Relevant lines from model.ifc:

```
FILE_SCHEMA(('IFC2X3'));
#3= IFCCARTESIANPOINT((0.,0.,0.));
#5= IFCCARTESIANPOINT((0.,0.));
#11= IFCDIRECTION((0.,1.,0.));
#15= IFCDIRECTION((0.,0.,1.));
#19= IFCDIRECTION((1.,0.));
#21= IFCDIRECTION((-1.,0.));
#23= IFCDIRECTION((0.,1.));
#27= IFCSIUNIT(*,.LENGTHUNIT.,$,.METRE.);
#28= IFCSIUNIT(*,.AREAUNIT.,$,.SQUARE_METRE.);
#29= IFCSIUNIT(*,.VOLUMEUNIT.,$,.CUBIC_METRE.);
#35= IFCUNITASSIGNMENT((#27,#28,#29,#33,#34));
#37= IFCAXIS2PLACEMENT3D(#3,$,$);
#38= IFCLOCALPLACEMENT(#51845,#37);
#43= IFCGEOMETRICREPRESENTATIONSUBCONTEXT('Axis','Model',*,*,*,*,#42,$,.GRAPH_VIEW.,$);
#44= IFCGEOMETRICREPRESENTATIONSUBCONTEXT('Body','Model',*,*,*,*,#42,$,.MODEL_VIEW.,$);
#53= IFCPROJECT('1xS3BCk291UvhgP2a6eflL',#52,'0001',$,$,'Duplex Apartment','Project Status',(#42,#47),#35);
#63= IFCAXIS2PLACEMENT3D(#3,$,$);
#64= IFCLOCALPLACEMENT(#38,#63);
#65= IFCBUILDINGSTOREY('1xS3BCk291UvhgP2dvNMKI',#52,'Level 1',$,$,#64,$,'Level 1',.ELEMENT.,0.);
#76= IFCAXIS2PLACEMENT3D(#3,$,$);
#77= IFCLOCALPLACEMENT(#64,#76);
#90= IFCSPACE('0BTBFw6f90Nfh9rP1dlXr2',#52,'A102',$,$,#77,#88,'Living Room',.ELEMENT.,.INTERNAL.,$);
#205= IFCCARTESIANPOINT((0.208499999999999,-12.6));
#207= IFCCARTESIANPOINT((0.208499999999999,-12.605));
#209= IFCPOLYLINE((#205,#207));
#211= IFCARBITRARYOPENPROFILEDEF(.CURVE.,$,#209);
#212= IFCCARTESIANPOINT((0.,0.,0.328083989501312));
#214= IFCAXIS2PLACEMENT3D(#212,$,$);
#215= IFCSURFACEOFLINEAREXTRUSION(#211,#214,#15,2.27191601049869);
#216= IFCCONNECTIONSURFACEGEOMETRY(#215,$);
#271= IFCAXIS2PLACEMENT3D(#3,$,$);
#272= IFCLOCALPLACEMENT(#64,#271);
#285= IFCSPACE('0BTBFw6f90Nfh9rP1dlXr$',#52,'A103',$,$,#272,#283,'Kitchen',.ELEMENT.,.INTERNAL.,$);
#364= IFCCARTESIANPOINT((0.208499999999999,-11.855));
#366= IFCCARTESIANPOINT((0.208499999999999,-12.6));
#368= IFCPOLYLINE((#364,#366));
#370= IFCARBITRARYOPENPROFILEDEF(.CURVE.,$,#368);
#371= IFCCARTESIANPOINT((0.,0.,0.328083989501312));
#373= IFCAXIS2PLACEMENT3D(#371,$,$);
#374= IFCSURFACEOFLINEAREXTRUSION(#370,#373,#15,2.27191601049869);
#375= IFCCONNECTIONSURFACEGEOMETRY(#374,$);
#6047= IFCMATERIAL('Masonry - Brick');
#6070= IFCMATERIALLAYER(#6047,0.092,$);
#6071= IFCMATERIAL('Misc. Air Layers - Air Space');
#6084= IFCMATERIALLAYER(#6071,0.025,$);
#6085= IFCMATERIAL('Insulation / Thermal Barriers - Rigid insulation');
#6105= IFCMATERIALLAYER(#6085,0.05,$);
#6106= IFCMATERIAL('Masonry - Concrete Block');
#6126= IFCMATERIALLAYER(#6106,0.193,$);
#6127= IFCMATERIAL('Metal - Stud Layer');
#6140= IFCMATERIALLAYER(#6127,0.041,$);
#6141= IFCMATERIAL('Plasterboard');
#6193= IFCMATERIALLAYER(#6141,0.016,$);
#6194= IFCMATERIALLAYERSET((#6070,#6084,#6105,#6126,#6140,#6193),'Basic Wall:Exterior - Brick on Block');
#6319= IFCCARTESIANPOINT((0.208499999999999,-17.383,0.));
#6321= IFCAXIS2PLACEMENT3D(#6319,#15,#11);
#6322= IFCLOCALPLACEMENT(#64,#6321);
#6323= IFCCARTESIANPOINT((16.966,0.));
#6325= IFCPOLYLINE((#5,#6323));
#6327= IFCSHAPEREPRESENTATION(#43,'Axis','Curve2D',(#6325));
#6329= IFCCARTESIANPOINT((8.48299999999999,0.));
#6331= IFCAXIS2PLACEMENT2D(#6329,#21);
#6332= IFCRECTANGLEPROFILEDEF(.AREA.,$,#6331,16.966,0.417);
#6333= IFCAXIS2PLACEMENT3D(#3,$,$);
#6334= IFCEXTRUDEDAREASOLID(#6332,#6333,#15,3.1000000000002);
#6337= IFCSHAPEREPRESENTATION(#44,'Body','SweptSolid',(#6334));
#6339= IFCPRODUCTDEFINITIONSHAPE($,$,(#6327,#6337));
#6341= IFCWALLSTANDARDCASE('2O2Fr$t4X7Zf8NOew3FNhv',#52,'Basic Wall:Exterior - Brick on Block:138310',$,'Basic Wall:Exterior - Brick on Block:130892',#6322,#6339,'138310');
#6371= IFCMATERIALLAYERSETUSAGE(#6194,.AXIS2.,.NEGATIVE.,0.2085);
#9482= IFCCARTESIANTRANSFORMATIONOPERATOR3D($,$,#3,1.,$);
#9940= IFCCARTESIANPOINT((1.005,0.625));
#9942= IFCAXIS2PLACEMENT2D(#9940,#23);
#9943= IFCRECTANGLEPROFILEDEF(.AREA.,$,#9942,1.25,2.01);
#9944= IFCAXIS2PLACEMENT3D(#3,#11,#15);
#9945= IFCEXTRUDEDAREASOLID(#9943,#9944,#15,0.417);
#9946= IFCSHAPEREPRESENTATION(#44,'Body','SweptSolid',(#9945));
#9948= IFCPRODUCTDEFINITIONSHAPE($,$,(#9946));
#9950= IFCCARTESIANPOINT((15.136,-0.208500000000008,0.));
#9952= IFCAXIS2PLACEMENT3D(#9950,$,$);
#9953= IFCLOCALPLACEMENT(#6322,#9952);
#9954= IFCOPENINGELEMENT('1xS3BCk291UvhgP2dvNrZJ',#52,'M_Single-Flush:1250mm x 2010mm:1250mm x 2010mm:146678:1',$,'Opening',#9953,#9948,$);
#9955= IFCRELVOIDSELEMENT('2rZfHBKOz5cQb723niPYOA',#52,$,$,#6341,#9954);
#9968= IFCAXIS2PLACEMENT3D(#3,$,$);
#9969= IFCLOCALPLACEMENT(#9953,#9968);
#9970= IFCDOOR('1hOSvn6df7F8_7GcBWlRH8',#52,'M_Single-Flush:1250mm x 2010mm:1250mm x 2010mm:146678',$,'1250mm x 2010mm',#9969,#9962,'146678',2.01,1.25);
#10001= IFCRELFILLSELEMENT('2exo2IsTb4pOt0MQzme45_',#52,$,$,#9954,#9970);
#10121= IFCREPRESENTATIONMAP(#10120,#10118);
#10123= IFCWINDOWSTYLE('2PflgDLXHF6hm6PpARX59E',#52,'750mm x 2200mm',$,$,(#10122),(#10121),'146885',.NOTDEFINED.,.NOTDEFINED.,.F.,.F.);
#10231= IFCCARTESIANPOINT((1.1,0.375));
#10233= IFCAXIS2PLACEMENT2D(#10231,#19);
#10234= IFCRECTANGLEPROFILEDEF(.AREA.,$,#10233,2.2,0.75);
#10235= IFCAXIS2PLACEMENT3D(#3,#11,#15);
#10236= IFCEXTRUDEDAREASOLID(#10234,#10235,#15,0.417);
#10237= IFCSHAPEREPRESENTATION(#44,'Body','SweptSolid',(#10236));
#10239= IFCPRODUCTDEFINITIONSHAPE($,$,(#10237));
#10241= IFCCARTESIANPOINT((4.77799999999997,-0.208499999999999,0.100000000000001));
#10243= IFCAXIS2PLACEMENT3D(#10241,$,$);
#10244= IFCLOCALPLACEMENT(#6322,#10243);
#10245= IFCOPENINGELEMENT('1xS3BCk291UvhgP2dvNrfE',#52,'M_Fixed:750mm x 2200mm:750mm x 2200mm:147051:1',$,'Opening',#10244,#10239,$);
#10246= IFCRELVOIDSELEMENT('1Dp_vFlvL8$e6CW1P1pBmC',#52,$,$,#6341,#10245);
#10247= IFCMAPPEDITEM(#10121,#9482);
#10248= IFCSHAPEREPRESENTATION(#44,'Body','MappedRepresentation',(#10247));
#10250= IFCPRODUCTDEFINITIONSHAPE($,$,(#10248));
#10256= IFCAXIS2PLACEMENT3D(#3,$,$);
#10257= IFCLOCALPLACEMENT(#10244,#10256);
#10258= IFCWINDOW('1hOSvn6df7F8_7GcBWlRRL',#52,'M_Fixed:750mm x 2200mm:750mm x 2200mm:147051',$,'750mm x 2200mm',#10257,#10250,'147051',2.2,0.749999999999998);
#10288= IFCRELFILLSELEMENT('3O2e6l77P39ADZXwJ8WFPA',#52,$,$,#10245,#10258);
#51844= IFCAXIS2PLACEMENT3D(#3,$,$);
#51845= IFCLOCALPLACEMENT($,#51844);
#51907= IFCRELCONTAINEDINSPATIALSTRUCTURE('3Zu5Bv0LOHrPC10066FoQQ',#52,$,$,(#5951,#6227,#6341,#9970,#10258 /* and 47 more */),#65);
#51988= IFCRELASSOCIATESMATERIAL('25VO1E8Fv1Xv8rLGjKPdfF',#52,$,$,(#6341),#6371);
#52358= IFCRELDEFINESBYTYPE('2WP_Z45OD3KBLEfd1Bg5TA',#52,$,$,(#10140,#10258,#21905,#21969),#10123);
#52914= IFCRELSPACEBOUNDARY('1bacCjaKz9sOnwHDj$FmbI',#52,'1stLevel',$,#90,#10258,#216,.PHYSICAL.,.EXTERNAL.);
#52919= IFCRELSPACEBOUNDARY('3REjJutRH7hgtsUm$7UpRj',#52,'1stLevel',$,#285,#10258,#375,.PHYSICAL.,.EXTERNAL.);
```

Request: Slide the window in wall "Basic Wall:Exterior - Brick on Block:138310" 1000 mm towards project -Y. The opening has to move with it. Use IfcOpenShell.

```python
import numpy as np
import ifcopenshell
import ifcopenshell.api.geometry
import ifcopenshell.util.placement
import ifcopenshell.util.unit

model = ifcopenshell.open("model.ifc")
unit_scale = ifcopenshell.util.unit.calculate_unit_scale(model)

window = model.by_guid("1hOSvn6df7F8_7GcBWlRRL")
opening = window.FillsVoids[0].RelatingOpeningElement
wall = opening.VoidsElements[0].RelatingBuildingElement

wall_matrix = ifcopenshell.util.placement.get_local_placement(wall.ObjectPlacement)
shift = wall_matrix[:3, 0] * -1 / unit_scale
before = ifcopenshell.util.placement.get_local_placement(window.ObjectPlacement)[:3, 3].copy()

# The window is placed relative to its opening, so it follows when the opening moves.
matrix = ifcopenshell.util.placement.get_local_placement(opening.ObjectPlacement)
matrix[:3, 3] += shift
ifcopenshell.api.geometry.edit_object_placement(
    model, product=opening, matrix=matrix, is_si=False, should_transform_children=True
)

# Space boundary surfaces are stored in each space's coordinates; move them too.
for rel in window.ProvidesBoundaries:
    if not rel.ConnectionGeometry:
        continue
    surface = rel.ConnectionGeometry.SurfaceOnRelatingElement
    space_matrix = ifcopenshell.util.placement.get_local_placement(rel.RelatingSpace.ObjectPlacement)
    point = np.array(surface.Position.Location.Coordinates) + space_matrix[:3, :3].T @ shift
    surface.Position = model.createIfcAxis2Placement3D(
        model.createIfcCartesianPoint(point.tolist()), surface.Position.Axis, surface.Position.RefDirection
    )

after = ifcopenshell.util.placement.get_local_placement(window.ObjectPlacement)[:3, 3]
print("window moved by", (after - before).round(3) + 0.0)

model.write("model_v2.ifc")
```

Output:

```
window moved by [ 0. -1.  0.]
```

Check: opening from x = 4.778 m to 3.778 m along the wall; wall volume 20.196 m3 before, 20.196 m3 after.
